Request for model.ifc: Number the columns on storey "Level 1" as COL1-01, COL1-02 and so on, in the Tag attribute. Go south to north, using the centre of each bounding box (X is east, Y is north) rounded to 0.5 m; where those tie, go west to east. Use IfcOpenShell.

First a look at what the model holds.

```python
import ifcopenshell
import ifcopenshell.util.element
import ifcopenshell.util.placement

model = ifcopenshell.open("model.ifc")
print(model.schema)
storey = next(s for s in model.by_type("IfcBuildingStorey") if s.Name == "Level 1")
columns = [e for e in ifcopenshell.util.element.get_decomposition(storey) if e.is_a("IfcColumn")]
for e in sorted(columns, key=lambda e: e.id()):
    origin = ifcopenshell.util.placement.get_local_placement(e.ObjectPlacement)[:3, 3]
    print(e.id(), e.Tag, e.Name, origin.round(2) + 0.0, sep=" | ")
```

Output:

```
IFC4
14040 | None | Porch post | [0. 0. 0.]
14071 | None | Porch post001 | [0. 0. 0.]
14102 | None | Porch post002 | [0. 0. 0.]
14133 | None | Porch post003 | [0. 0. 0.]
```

```python
import ifcopenshell
import ifcopenshell.geom
import ifcopenshell.util.element
import ifcopenshell.util.shape

model = ifcopenshell.open("model.ifc")
settings = ifcopenshell.geom.settings()
settings.set("use-world-coords", True)


def centre(element):
    shape = ifcopenshell.geom.create_shape(settings, element)
    return ifcopenshell.util.shape.get_bbox_centroid(shape.geometry)


storey = next(s for s in model.by_type("IfcBuildingStorey") if s.Name == "Level 1")
columns = [e for e in ifcopenshell.util.element.get_decomposition(storey) if e.is_a("IfcColumn")]

# Insertion points can sit at a corner or the storey origin, so sort by the geometry (in metres).
centres = {e: centre(e) for e in columns}
columns.sort(key=lambda e: (round(centres[e][1] / 0.5), centres[e][0]))

for i, e in enumerate(columns, start=1):
    number = f"COL1-{i:02d}"
    e.Tag = number
    print(e.id(), number)

model.write("model_rev.ifc")
```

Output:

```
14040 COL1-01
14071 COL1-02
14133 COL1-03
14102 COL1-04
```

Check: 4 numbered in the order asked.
